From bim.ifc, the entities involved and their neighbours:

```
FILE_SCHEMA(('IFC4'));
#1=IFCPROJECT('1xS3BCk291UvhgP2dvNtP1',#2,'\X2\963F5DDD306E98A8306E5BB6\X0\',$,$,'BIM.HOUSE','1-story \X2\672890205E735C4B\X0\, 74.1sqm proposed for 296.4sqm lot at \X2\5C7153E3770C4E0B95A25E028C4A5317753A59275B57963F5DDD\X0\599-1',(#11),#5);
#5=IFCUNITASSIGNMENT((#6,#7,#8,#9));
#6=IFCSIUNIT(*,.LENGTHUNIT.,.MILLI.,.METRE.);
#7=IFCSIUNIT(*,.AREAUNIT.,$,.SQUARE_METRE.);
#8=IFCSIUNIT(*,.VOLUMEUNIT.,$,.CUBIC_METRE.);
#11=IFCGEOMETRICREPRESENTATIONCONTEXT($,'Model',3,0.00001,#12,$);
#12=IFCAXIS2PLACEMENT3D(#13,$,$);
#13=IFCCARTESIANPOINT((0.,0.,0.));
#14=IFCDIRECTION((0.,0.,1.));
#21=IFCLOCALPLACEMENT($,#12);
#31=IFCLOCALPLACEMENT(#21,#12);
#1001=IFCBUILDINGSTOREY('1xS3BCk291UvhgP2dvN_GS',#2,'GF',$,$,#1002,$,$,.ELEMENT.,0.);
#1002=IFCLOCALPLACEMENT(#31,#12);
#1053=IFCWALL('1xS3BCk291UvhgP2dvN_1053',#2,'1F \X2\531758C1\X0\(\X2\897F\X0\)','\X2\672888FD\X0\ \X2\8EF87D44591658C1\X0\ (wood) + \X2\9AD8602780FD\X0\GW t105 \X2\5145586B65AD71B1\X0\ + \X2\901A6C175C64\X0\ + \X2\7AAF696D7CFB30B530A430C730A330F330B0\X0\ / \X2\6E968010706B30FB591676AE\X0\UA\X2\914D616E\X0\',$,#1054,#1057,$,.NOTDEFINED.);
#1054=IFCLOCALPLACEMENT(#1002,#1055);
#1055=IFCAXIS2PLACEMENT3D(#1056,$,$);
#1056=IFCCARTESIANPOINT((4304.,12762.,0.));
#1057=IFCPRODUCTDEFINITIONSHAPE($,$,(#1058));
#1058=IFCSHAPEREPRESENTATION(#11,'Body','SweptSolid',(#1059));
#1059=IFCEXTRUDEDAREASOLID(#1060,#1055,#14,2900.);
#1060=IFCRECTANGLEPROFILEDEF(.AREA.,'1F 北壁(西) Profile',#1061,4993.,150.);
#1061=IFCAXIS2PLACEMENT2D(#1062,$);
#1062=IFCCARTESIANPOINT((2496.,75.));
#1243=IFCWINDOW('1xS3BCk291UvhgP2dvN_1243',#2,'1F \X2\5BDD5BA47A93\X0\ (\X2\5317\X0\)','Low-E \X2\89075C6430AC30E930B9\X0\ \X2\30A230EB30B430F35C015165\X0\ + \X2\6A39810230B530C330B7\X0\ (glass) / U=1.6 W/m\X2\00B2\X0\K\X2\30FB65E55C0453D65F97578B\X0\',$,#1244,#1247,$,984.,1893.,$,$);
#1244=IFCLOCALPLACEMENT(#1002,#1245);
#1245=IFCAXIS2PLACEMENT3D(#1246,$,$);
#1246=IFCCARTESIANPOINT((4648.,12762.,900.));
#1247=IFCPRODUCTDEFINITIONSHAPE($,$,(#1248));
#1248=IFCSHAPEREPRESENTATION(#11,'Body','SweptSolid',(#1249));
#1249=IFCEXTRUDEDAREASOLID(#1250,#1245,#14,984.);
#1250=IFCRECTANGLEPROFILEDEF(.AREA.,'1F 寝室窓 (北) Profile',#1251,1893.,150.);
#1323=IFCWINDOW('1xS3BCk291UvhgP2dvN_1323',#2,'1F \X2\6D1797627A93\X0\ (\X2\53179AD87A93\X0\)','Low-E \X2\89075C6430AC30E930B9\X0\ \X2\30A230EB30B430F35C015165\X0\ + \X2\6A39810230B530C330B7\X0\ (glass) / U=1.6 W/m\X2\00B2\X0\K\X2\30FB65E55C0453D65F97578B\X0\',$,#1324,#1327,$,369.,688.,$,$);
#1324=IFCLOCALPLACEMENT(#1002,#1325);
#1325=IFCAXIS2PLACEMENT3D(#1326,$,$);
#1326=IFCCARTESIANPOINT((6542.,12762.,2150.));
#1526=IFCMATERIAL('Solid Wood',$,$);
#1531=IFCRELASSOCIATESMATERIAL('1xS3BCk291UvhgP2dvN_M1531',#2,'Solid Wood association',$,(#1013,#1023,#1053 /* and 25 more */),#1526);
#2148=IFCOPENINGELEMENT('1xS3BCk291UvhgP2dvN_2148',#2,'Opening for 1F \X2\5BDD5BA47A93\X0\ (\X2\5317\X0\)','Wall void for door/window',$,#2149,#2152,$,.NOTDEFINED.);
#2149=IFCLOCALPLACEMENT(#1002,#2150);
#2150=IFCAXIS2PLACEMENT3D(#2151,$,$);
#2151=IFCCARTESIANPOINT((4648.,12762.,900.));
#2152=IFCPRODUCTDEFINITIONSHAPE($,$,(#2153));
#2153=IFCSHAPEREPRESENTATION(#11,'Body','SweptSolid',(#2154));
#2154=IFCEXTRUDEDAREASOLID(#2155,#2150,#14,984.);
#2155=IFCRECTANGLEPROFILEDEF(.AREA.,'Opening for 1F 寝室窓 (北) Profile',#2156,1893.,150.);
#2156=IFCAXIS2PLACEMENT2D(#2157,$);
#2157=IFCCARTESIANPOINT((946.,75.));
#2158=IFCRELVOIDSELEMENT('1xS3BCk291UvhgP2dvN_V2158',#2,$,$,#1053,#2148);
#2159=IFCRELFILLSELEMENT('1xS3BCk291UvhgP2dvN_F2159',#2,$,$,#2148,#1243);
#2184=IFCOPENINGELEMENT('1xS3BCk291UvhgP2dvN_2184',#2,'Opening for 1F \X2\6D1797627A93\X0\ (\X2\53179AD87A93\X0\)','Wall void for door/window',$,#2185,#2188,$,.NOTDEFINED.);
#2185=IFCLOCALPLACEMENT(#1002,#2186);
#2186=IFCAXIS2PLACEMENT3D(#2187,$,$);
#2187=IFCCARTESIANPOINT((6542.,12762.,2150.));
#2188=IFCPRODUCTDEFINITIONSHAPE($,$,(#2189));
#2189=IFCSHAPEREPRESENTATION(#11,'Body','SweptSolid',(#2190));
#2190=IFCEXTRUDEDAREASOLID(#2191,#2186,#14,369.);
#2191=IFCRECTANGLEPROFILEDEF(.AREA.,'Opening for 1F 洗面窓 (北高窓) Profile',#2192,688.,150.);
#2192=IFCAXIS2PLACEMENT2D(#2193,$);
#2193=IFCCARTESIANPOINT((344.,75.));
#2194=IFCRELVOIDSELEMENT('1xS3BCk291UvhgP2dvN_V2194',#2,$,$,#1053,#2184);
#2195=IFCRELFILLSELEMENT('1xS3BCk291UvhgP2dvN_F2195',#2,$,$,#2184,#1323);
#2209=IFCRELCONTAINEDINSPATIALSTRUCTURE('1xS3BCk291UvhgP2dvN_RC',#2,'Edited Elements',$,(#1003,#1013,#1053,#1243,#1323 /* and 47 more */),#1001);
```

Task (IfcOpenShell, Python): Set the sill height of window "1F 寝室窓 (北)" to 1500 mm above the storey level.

```python
import numpy as np
import ifcopenshell
import ifcopenshell.api.geometry
import ifcopenshell.geom
import ifcopenshell.util.element
import ifcopenshell.util.placement
import ifcopenshell.util.shape
import ifcopenshell.util.unit

model = ifcopenshell.open("bim.ifc")
unit_scale = ifcopenshell.util.unit.calculate_unit_scale(model)

window = model.by_id(1243)
opening = window.FillsVoids[0].RelatingOpeningElement
storey = ifcopenshell.util.element.get_container(window, ifc_class="IfcBuildingStorey")
level = ifcopenshell.util.placement.get_local_placement(storey.ObjectPlacement)[2, 3]

# The opening's origin need not be at the sill, so measure its lowest point.
shape = ifcopenshell.geom.create_shape(ifcopenshell.geom.settings(), opening)
bottom = ifcopenshell.util.shape.get_shape_bottom_elevation(shape, shape.geometry) / unit_scale
dz = level + 1500.0 - bottom

shift = np.array([0.0, 0.0, dz])
# The window is not placed relative to its opening, so move both.
for product in (opening, window):
    matrix = ifcopenshell.util.placement.get_local_placement(product.ObjectPlacement)
    matrix[:3, 3] += shift
    ifcopenshell.api.geometry.edit_object_placement(model, product=product, matrix=matrix, is_si=False)

print(f"moved by {dz * unit_scale:+.3f} m")

model.write("bim_updated.ifc")
```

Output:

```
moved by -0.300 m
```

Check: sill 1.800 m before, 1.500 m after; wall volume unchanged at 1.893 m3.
